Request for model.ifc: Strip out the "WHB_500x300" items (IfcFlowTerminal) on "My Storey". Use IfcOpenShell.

First a look at what the model holds.

```python
import ifcopenshell
import ifcopenshell.util.element

model = ifcopenshell.open("model.ifc")
print(model.schema)
storey = next(s for s in model.by_type("IfcBuildingStorey") if s.Name == "My Storey")
terminals = [e for e in ifcopenshell.util.element.get_decomposition(storey) if e.is_a("IfcFlowTerminal")]
seen = {}
for e in terminals:
    element_type = ifcopenshell.util.element.get_type(e)
    name = element_type.Name if element_type not in (None, e) else None
    seen[name] = seen.get(name, 0) + 1
for name, count in sorted(seen.items(), key=str):
    print(count, "x", name)
```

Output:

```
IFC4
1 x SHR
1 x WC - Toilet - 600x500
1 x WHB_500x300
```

```python
import ifcopenshell
import ifcopenshell.api.root
import ifcopenshell.util.element

model = ifcopenshell.open("model.ifc")

storey = next(s for s in model.by_type("IfcBuildingStorey") if s.Name == "My Storey")
terminals = [e for e in ifcopenshell.util.element.get_decomposition(storey) if e.is_a("IfcFlowTerminal")]
targets = [e for e in terminals if (t := ifcopenshell.util.element.get_type(e)) not in (None, e) and t.Name == "WHB_500x300"]

for e in targets:
    ifcopenshell.api.root.remove_product(model, product=e)
print(len(targets), "removed")

model.write("model_v2.ifc")
```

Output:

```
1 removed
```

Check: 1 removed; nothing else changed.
